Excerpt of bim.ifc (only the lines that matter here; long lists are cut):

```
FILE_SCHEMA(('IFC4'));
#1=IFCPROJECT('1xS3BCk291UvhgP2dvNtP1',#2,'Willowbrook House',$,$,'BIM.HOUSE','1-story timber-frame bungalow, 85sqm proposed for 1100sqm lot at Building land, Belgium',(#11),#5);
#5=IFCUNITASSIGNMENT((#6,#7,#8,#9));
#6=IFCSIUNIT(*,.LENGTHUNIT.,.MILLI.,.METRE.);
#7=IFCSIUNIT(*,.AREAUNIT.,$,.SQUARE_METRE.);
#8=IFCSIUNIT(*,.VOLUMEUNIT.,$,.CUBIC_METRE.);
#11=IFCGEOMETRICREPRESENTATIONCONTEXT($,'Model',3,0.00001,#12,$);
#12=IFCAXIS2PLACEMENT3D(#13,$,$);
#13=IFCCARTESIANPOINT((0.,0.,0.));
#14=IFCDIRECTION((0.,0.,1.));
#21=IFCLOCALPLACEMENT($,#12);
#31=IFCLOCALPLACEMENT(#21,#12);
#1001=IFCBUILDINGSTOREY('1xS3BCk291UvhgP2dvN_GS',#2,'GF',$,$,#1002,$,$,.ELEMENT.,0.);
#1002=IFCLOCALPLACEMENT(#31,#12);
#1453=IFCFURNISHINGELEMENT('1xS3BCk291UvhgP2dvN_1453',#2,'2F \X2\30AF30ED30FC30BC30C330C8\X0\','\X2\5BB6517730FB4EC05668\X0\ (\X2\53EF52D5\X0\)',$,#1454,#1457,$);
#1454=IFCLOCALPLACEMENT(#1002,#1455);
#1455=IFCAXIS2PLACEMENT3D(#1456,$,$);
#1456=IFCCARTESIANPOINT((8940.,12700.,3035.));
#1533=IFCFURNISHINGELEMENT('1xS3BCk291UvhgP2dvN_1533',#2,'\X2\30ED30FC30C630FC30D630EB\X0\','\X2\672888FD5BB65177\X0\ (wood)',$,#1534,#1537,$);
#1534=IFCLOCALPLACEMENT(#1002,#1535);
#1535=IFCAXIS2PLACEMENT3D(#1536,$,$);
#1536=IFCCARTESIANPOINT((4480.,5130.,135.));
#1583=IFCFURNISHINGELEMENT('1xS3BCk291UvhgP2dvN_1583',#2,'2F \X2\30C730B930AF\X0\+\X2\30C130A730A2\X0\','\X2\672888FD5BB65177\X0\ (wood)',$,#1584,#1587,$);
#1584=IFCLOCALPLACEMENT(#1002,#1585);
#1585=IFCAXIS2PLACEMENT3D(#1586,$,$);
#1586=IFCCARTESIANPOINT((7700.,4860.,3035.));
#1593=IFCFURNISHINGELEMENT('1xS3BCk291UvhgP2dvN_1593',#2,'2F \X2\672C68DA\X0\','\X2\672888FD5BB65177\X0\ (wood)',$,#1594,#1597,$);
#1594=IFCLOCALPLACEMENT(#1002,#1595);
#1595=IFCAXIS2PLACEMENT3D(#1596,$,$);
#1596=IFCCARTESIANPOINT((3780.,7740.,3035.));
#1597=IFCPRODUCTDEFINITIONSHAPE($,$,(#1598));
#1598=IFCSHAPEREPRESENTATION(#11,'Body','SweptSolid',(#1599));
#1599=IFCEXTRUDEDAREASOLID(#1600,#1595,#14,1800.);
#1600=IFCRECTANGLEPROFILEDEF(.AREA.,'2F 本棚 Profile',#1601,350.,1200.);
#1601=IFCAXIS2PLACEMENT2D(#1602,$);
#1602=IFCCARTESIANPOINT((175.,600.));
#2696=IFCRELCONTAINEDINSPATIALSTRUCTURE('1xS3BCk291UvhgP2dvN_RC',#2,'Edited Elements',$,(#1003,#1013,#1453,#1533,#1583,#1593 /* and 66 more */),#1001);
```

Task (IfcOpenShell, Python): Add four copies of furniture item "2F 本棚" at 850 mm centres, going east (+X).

```python
import numpy as np
import ifcopenshell
import ifcopenshell.api.geometry
import ifcopenshell.api.root
import ifcopenshell.util.element
import ifcopenshell.util.placement
import ifcopenshell.util.unit

model = ifcopenshell.open("bim.ifc")
unit_scale = ifcopenshell.util.unit.calculate_unit_scale(model)


def reuse_history(source, copy):
    """copy_class also copies each property set's owner history, people and application; keep the originals."""
    for rel in copy.IsDefinedBy:
        if rel.is_a("IfcRelDefinesByProperties") and (history := rel.RelatingPropertyDefinition.OwnerHistory):
            rel.RelatingPropertyDefinition.OwnerHistory = source.OwnerHistory
            ifcopenshell.util.element.remove_deep2(model, history)


source = model.by_guid("1xS3BCk291UvhgP2dvN_1593")
base = ifcopenshell.util.placement.get_local_placement(source.ObjectPlacement)
step = np.array([1.0, 0.0, 0.0]) * 0.85 / unit_scale

for i in range(1, 5):
    copy = ifcopenshell.api.root.copy_class(model, product=source)
    copy.Representation = ifcopenshell.util.element.copy_deep(
        model, source.Representation, exclude=["IfcGeometricRepresentationContext", "IfcRepresentationMap"]
    )
    reuse_history(source, copy)
    matrix = base.copy()
    matrix[:3, 3] += i * step
    print("added at", matrix[:3, 3].round(3) + 0.0)
    ifcopenshell.api.geometry.edit_object_placement(model, product=copy, matrix=matrix, is_si=False)

model.write("bim_edited.ifc")
```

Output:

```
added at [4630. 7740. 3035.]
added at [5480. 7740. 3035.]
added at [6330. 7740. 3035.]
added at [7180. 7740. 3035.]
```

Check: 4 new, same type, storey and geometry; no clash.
